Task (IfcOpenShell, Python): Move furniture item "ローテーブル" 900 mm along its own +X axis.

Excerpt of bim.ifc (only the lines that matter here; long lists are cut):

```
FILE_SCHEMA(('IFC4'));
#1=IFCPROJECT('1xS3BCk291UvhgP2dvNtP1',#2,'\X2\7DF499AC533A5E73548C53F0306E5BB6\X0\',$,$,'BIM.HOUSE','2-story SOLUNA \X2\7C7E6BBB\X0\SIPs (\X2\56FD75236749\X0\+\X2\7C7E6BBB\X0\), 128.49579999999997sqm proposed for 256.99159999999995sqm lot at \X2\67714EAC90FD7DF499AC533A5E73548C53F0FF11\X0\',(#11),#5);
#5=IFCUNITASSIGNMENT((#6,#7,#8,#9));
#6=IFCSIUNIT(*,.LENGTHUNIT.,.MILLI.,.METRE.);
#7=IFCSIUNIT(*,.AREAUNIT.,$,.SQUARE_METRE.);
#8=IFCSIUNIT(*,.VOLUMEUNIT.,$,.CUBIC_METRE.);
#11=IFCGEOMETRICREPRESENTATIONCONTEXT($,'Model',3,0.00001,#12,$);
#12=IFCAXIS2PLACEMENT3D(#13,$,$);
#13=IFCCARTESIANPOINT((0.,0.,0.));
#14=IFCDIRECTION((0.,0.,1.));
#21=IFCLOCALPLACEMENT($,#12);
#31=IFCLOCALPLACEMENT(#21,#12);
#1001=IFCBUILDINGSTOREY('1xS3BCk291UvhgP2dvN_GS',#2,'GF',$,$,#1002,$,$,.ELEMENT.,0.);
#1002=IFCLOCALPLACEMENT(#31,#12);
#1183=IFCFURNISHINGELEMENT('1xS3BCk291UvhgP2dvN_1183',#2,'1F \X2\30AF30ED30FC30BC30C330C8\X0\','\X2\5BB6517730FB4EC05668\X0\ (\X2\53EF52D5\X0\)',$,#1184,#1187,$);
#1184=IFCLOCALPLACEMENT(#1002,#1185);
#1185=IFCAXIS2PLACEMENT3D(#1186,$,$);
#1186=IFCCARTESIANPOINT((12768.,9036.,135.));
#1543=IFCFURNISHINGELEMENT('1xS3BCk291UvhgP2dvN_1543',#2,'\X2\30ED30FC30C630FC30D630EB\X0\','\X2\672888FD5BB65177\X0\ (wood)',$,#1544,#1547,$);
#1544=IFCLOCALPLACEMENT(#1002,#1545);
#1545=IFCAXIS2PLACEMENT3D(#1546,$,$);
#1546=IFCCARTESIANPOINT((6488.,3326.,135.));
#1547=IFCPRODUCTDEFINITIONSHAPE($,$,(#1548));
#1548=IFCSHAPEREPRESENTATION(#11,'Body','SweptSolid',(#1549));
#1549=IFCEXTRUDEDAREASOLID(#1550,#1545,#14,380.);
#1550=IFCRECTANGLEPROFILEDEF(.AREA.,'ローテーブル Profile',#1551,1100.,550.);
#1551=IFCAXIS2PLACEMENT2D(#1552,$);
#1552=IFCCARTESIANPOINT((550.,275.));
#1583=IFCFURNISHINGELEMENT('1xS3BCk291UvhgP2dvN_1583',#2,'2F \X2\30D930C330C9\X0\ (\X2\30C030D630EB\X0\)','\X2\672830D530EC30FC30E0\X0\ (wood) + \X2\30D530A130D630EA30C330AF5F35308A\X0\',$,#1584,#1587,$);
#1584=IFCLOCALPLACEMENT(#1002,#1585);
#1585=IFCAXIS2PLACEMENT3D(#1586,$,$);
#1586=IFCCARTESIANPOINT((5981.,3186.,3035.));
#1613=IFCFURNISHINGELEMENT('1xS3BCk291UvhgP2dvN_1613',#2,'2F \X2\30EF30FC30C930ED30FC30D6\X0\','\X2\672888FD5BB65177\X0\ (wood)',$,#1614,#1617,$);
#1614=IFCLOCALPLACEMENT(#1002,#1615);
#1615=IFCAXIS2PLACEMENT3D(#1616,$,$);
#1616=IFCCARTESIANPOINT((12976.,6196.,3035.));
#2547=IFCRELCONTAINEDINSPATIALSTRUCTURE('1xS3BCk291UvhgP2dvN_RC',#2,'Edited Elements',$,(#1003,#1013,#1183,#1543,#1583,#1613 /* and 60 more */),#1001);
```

```python
import ifcopenshell
import ifcopenshell.api.geometry
import ifcopenshell.util.placement

model = ifcopenshell.open("bim.ifc")

item = model.by_id(1543)
matrix = ifcopenshell.util.placement.get_local_placement(item.ObjectPlacement)
matrix[:3, 3] += matrix[:3, 0] * 900.0
ifcopenshell.api.geometry.edit_object_placement(model, product=item, matrix=matrix, is_si=False)

print(ifcopenshell.util.placement.get_local_placement(item.ObjectPlacement).round(3) + 0.0)

model.write("bim_rev.ifc")
```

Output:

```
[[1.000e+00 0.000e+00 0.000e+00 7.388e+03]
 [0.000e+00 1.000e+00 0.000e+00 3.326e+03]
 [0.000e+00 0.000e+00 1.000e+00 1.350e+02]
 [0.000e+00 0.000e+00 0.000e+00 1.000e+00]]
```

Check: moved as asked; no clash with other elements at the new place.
